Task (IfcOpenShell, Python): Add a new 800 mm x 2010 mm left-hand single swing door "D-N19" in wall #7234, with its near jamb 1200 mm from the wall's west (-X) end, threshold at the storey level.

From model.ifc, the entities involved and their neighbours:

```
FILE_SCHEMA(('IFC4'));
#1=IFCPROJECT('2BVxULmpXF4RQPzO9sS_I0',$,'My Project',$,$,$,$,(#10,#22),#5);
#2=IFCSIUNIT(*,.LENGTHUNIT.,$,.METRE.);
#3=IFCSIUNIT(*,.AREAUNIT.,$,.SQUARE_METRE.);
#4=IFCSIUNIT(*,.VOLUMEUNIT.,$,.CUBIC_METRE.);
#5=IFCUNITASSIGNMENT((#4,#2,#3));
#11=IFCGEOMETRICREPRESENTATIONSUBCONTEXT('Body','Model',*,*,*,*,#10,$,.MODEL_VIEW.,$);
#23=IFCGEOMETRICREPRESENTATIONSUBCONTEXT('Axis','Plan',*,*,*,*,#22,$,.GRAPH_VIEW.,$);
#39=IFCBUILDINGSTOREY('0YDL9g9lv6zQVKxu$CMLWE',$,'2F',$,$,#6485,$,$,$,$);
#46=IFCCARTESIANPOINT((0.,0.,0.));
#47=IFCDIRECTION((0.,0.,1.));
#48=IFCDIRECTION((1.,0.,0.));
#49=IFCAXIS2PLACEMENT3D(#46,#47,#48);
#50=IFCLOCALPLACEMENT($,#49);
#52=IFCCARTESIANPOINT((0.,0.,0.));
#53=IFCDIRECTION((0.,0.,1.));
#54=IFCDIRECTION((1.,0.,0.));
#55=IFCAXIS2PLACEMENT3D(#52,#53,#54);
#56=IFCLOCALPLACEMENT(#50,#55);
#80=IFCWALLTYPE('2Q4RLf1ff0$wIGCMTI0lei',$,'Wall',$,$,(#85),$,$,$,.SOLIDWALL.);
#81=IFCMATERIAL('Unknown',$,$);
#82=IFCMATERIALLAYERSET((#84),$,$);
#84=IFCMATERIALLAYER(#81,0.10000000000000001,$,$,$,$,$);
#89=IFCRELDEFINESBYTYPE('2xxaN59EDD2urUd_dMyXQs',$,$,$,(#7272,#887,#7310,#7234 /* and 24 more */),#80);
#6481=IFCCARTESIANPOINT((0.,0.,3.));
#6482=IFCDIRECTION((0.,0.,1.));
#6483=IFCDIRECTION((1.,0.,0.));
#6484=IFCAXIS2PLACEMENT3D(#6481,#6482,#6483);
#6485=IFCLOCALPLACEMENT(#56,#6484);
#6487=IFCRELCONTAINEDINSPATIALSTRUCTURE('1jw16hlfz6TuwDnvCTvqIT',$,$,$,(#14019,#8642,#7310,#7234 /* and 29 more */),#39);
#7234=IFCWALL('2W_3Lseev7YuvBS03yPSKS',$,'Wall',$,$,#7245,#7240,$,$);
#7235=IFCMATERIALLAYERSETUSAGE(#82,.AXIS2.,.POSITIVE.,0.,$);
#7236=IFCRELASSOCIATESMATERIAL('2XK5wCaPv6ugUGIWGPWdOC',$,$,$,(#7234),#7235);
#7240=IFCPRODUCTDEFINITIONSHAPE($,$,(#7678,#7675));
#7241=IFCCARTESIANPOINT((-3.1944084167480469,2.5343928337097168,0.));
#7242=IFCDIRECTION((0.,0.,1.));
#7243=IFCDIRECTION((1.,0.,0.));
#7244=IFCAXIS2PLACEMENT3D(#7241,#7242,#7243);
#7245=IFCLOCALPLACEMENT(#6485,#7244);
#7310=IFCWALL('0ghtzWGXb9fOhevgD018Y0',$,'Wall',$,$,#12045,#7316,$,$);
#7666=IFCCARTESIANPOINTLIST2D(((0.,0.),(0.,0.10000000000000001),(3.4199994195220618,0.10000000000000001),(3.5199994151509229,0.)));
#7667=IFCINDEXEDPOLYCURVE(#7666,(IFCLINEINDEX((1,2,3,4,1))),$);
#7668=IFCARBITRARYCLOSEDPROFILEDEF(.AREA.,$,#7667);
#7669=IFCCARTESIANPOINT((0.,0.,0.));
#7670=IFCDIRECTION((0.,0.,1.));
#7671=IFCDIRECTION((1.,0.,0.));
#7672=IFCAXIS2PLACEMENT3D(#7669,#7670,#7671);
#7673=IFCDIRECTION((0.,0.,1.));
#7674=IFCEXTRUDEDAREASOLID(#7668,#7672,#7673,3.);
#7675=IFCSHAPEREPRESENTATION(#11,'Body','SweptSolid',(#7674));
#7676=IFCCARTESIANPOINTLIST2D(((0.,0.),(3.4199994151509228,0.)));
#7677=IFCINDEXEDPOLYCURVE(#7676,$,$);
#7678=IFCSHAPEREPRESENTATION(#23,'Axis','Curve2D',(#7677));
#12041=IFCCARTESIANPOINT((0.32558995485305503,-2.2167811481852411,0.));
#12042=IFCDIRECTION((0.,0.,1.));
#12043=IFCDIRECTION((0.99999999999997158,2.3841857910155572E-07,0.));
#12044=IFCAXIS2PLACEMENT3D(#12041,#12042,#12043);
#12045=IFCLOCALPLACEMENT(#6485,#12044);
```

```python
import numpy as np
import ifcopenshell
import ifcopenshell.api.feature
import ifcopenshell.api.geometry
import ifcopenshell.api.root
import ifcopenshell.api.spatial
import ifcopenshell.geom
import ifcopenshell.util.element
import ifcopenshell.util.placement
import ifcopenshell.util.representation
import ifcopenshell.util.shape
import ifcopenshell.util.unit

model = ifcopenshell.open("model.ifc")
unit_scale = ifcopenshell.util.unit.calculate_unit_scale(model)
settings = ifcopenshell.geom.settings()


def volume(element):
    """Net volume in cubic metres, openings subtracted."""
    shape = ifcopenshell.geom.create_shape(settings, element)
    return ifcopenshell.util.shape.get_volume(shape.geometry)


wall = model.by_guid("2W_3Lseev7YuvBS03yPSKS")
storey = ifcopenshell.util.element.get_container(wall, ifc_class="IfcBuildingStorey")
context = ifcopenshell.util.representation.get_context(model, "Model", "Body", "MODEL_VIEW")
before = volume(wall)

width, height, from_end, sill = 0.8, 2.01, 1.2, 0.0  # metres

# The wall runs along its own X axis, and the end named is its -X end.
wall_shape = ifcopenshell.geom.create_shape(settings, wall)
x, y, z = ifcopenshell.util.shape.get_vertices(wall_shape.geometry).T
start = x.min() + from_end
face, thickness = float(y.min()), float(y.max() - y.min())
wall_matrix = ifcopenshell.util.placement.get_local_placement(wall.ObjectPlacement)
level = ifcopenshell.util.placement.get_local_placement(storey.ObjectPlacement)[2, 3]


def in_wall(x, y):
    """Placement at x, y metres in the wall's axes, at sill height."""
    matrix = wall_matrix.copy()
    matrix[:, 3] = wall_matrix @ np.array([x / unit_scale, y / unit_scale, 0.0, 1.0])
    matrix[2, 3] = level + sill / unit_scale
    return matrix


# Opening: a box that overshoots both wall faces by 50 mm.
opening = ifcopenshell.api.root.create_entity(model, ifc_class="IfcOpeningElement", predefined_type="OPENING")
box = ifcopenshell.api.geometry.add_wall_representation(
    model, context=context, length=width, height=height, thickness=thickness + 0.1
)
ifcopenshell.api.geometry.assign_representation(model, product=opening, representation=box)
ifcopenshell.api.geometry.edit_object_placement(model, product=opening, matrix=in_wall(start, face - 0.05), is_si=False)
ifcopenshell.api.feature.add_feature(model, feature=opening, element=wall)

door = ifcopenshell.api.root.create_entity(model, ifc_class="IfcDoor", name="D-N19", predefined_type="DOOR")
door.OverallWidth, door.OverallHeight = width / unit_scale, height / unit_scale
door.OperationType = "SINGLE_SWING_LEFT"
body = ifcopenshell.api.geometry.add_door_representation(
    model,
    context=context,
    overall_width=door.OverallWidth,
    overall_height=door.OverallHeight,
    operation_type="SINGLE_SWING_LEFT",
    lining_properties={"LiningDepth": thickness / unit_scale, "ThresholdDepth": thickness / unit_scale},
)
ifcopenshell.api.geometry.assign_representation(model, product=door, representation=body)
ifcopenshell.api.spatial.assign_container(model, products=[door], relating_structure=storey)
ifcopenshell.api.feature.add_filling(model, opening=opening, element=door)

# The lining spans the wall, so the door starts at the wall face.
ifcopenshell.api.geometry.edit_object_placement(model, product=door, matrix=in_wall(start, face), is_si=False)

after = volume(wall)

print(f"wall volume {before:.3f} -> {after:.3f} m3")

model.write("model_v2.ifc")
```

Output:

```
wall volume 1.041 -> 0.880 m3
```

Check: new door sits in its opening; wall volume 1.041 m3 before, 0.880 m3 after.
